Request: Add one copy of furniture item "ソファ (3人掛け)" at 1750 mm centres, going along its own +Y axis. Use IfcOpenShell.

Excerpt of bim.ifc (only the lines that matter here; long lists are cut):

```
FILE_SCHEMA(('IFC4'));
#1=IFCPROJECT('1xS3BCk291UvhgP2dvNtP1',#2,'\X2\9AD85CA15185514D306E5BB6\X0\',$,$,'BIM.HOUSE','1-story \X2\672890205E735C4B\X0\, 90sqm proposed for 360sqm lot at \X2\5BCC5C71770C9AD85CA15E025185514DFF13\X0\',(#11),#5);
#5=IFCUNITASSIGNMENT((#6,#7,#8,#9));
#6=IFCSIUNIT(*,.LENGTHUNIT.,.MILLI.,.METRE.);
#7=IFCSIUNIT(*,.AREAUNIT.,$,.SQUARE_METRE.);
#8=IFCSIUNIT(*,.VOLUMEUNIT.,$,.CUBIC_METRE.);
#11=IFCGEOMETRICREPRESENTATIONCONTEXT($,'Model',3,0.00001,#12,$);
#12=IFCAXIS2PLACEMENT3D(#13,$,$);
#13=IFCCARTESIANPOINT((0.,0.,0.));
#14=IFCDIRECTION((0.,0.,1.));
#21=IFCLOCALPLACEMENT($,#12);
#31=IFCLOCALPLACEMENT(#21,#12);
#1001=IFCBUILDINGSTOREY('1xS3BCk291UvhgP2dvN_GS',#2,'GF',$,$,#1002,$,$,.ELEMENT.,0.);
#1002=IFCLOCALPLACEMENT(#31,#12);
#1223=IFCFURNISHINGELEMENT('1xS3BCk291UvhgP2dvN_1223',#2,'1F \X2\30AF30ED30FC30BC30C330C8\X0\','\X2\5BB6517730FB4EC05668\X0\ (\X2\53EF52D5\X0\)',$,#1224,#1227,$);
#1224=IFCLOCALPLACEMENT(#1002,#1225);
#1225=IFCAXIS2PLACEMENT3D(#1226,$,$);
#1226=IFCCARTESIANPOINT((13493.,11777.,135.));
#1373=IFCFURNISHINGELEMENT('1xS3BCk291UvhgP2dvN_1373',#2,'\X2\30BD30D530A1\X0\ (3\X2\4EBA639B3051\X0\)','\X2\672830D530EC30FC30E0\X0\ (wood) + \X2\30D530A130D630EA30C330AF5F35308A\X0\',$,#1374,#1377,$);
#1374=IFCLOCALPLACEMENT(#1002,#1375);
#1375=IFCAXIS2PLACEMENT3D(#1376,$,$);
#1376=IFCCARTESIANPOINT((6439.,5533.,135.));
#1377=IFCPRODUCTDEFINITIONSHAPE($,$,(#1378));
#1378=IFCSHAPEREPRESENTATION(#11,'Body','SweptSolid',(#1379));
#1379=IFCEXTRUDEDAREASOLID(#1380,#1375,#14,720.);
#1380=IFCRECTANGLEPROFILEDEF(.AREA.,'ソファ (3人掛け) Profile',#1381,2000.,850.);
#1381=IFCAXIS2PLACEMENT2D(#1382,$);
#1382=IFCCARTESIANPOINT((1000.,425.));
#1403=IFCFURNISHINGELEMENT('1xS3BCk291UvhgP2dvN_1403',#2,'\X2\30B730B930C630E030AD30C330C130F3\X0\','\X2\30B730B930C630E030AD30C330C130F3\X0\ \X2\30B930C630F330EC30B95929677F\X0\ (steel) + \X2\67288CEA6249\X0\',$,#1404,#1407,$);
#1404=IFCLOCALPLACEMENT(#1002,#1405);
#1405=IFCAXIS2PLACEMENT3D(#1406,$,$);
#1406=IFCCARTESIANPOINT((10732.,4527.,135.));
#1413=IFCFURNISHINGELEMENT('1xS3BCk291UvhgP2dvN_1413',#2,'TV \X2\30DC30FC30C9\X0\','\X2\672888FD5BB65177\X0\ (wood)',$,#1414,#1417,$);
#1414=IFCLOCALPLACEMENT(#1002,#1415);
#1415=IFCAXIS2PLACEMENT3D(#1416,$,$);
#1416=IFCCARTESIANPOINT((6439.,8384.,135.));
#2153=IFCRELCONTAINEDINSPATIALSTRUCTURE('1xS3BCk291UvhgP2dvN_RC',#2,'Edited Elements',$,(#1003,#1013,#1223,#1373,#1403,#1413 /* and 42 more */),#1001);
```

```python
import ifcopenshell
import ifcopenshell.api.geometry
import ifcopenshell.api.root
import ifcopenshell.util.element
import ifcopenshell.util.placement
import ifcopenshell.util.unit

model = ifcopenshell.open("bim.ifc")
unit_scale = ifcopenshell.util.unit.calculate_unit_scale(model)


def reuse_history(source, copy):
    """copy_class also copies each property set's owner history, people and application; keep the originals."""
    for rel in copy.IsDefinedBy:
        if rel.is_a("IfcRelDefinesByProperties") and (history := rel.RelatingPropertyDefinition.OwnerHistory):
            rel.RelatingPropertyDefinition.OwnerHistory = source.OwnerHistory
            ifcopenshell.util.element.remove_deep2(model, history)


source = model.by_guid("1xS3BCk291UvhgP2dvN_1373")
base = ifcopenshell.util.placement.get_local_placement(source.ObjectPlacement)
step = base[:3, 1] * 1.75 / unit_scale

for i in range(1, 2):
    copy = ifcopenshell.api.root.copy_class(model, product=source)
    copy.Representation = ifcopenshell.util.element.copy_deep(
        model, source.Representation, exclude=["IfcGeometricRepresentationContext", "IfcRepresentationMap"]
    )
    reuse_history(source, copy)
    matrix = base.copy()
    matrix[:3, 3] += i * step
    print("added at", matrix[:3, 3].round(3) + 0.0)
    ifcopenshell.api.geometry.edit_object_placement(model, product=copy, matrix=matrix, is_si=False)

model.write("bim_v2.ifc")
```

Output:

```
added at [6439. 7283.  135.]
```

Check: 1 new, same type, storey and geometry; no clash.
